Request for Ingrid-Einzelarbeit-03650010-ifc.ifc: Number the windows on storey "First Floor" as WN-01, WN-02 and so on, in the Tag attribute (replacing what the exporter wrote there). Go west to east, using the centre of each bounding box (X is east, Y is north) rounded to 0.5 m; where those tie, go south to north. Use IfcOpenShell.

First a look at what the model holds.

```python
import ifcopenshell
import ifcopenshell.util.element
import ifcopenshell.util.placement

model = ifcopenshell.open("Ingrid-Einzelarbeit-03650010-ifc.ifc")
print(model.schema)
storey = next(s for s in model.by_type("IfcBuildingStorey") if s.Name == "First Floor")
windows = [e for e in ifcopenshell.util.element.get_decomposition(storey) if e.is_a("IfcWindow")]
for e in sorted(windows, key=lambda e: e.id()):
    origin = ifcopenshell.util.placement.get_local_placement(e.ObjectPlacement)[:3, 3]
    print(e.id(), e.Tag, e.Name, origin.round(2) + 0.0, sep=" | ")
```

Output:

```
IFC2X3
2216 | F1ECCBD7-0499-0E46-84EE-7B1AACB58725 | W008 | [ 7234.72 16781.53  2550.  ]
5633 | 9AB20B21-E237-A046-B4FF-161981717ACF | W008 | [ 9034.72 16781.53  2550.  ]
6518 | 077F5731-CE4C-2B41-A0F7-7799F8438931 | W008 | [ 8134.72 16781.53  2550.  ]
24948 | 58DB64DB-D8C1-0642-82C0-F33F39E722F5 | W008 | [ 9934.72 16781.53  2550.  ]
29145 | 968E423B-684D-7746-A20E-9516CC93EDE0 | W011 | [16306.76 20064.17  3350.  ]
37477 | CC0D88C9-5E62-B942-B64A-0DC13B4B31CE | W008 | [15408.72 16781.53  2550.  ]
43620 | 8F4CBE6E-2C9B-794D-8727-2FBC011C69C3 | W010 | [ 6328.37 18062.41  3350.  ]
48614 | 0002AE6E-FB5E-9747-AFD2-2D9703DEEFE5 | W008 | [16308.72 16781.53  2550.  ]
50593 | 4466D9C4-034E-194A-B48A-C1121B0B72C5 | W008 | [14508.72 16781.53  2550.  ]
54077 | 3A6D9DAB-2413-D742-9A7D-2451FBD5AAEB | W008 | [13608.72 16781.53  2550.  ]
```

```python
import ifcopenshell
import ifcopenshell.geom
import ifcopenshell.util.element
import ifcopenshell.util.shape

model = ifcopenshell.open("Ingrid-Einzelarbeit-03650010-ifc.ifc")
settings = ifcopenshell.geom.settings()
settings.set("use-world-coords", True)


def centre(element):
    shape = ifcopenshell.geom.create_shape(settings, element)
    return ifcopenshell.util.shape.get_bbox_centroid(shape.geometry)


storey = next(s for s in model.by_type("IfcBuildingStorey") if s.Name == "First Floor")
windows = [e for e in ifcopenshell.util.element.get_decomposition(storey) if e.is_a("IfcWindow")]

# Insertion points can sit at a corner or the storey origin, so sort by the geometry (in metres).
centres = {e: centre(e) for e in windows}
windows.sort(key=lambda e: (round(centres[e][0] / 0.5), centres[e][1]))

for i, e in enumerate(windows, start=1):
    number = f"WN-{i:02d}"
    e.Tag = number
    print(e.id(), number)

model.write("Ingrid-Einzelarbeit-03650010-ifc_rev.ifc")
```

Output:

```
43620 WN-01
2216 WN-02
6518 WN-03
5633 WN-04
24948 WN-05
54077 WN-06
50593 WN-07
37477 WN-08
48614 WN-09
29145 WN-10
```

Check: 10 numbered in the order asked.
